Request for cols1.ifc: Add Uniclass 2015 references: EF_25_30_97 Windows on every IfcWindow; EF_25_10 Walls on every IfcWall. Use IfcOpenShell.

First a look at what the model holds.

```python
import ifcopenshell

model = ifcopenshell.open("cols1.ifc")
print(model.schema)
print("classifications:", [c.Name for c in model.by_type("IfcClassification")])
for ifc_class in ("IfcDoor", "IfcRoof", "IfcStair", "IfcWall", "IfcWindow"):
    print(ifc_class, len(model.by_type(ifc_class)))
```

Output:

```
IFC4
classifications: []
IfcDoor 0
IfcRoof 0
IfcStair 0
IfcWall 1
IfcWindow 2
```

```python
import ifcopenshell
import ifcopenshell.api.classification

model = ifcopenshell.open("cols1.ifc")

system = ifcopenshell.api.classification.add_classification(model, classification="Uniclass 2015")

codes = {
    "IfcWindow": ("EF_25_30_97", "Windows"),
    "IfcWall": ("EF_25_10", "Walls"),
}
for ifc_class, (code, name) in codes.items():
    products = model.by_type(ifc_class)
    ifcopenshell.api.classification.add_reference(
        model, products=products, classification=system, identification=code, name=name
    )
    print(code, len(products))

model.write("cols1_rev.ifc")
```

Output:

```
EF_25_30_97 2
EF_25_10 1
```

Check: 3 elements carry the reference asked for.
